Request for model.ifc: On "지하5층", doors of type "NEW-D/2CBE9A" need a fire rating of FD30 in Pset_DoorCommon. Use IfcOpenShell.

First a look at what the model holds.

```python
import ifcopenshell
import ifcopenshell.util.element

model = ifcopenshell.open("model.ifc")
print(model.schema)
storey = next(s for s in model.by_type("IfcBuildingStorey") if s.Name == "지하5층")
doors = [e for e in ifcopenshell.util.element.get_decomposition(storey) if e.is_a("IfcDoor")]
seen = {}
for e in doors:
    element_type = ifcopenshell.util.element.get_type(e)
    key = (element_type.Name if element_type != e and element_type else None, ifcopenshell.util.element.get_pset(e, "Pset_DoorCommon", "FireRating"))
    seen[key] = seen.get(key, 0) + 1
for (name, value), count in sorted(seen.items(), key=str):
    print(count, "x", name, "|", value)
```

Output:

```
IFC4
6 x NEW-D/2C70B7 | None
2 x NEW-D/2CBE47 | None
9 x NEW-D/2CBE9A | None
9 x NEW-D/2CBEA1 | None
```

```python
import ifcopenshell
import ifcopenshell.api.pset
import ifcopenshell.util.element

model = ifcopenshell.open("model.ifc")

storey = next(s for s in model.by_type("IfcBuildingStorey") if s.Name == "지하5층")
doors = [e for e in ifcopenshell.util.element.get_decomposition(storey) if e.is_a("IfcDoor")]

count = 0
for e in doors:
    element_type = ifcopenshell.util.element.get_type(e)
    if element_type in (None, e) or element_type.Name != "NEW-D/2CBE9A":
        continue
    # add_pset returns the element's existing set when there is one.
    pset = ifcopenshell.api.pset.add_pset(model, product=e, name="Pset_DoorCommon")
    ifcopenshell.api.pset.edit_pset(model, pset=pset, properties={"FireRating": "FD30"})
    count += 1

print(count, "doors updated")

model.write("model-out.ifc")
```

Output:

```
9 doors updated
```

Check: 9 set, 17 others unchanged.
